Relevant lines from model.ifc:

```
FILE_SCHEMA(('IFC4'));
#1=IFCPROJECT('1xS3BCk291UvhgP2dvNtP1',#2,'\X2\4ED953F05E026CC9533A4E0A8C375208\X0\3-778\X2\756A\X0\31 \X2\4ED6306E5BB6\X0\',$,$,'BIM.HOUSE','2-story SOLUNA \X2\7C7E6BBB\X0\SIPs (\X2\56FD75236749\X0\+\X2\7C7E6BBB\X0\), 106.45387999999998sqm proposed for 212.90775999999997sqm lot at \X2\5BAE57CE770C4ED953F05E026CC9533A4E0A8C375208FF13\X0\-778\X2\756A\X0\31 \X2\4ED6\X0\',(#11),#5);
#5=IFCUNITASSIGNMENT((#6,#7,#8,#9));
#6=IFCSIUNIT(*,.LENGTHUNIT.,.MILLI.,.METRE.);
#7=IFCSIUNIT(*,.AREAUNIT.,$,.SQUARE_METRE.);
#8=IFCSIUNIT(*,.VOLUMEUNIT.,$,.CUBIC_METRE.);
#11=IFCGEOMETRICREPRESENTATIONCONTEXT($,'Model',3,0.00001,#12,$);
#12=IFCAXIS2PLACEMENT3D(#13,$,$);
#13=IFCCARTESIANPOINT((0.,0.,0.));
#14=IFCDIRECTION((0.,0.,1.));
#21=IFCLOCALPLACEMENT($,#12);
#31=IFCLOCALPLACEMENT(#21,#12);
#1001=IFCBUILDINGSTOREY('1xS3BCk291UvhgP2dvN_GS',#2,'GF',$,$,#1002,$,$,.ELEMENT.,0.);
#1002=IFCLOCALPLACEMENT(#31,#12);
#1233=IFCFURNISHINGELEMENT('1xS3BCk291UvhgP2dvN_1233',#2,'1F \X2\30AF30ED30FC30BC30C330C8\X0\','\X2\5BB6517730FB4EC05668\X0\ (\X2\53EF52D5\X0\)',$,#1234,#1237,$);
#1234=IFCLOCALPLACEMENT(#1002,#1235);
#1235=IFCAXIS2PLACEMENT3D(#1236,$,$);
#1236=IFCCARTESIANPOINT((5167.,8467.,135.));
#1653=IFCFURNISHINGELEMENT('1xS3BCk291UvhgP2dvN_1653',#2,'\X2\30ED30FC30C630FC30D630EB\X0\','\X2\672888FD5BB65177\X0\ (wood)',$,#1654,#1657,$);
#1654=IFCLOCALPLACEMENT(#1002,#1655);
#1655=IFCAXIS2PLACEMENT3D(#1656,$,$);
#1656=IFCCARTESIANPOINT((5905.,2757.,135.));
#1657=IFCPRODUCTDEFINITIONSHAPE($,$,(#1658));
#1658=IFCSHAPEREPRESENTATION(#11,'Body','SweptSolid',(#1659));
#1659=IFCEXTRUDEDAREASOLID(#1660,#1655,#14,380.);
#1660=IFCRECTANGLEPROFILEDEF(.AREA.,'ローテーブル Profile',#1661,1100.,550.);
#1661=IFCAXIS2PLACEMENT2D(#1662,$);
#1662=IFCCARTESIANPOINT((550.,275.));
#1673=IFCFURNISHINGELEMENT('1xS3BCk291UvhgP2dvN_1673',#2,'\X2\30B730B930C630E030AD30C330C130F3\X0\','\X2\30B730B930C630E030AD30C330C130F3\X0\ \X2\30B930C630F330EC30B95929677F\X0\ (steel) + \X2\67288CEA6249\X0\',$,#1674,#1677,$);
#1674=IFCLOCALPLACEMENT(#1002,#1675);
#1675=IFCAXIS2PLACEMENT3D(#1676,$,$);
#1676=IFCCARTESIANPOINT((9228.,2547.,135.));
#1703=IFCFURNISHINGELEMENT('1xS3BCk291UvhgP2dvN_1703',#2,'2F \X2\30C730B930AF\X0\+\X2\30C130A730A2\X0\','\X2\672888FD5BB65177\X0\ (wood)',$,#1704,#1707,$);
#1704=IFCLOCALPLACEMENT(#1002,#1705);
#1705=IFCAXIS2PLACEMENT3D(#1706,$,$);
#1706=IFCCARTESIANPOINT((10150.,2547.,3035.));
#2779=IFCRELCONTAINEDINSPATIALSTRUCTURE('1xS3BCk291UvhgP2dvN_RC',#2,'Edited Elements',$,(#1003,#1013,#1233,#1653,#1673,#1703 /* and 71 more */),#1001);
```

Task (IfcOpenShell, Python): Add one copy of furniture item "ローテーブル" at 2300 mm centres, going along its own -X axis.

```python
import ifcopenshell
import ifcopenshell.api.geometry
import ifcopenshell.api.root
import ifcopenshell.util.element
import ifcopenshell.util.placement
import ifcopenshell.util.unit

model = ifcopenshell.open("model.ifc")
unit_scale = ifcopenshell.util.unit.calculate_unit_scale(model)


def reuse_history(source, copy):
    """copy_class also copies each property set's owner history, people and application; keep the originals."""
    for rel in copy.IsDefinedBy:
        if rel.is_a("IfcRelDefinesByProperties") and (history := rel.RelatingPropertyDefinition.OwnerHistory):
            rel.RelatingPropertyDefinition.OwnerHistory = source.OwnerHistory
            ifcopenshell.util.element.remove_deep2(model, history)


source = model.by_guid("1xS3BCk291UvhgP2dvN_1653")
base = ifcopenshell.util.placement.get_local_placement(source.ObjectPlacement)
step = -base[:3, 0] * 2.3 / unit_scale

for i in range(1, 2):
    copy = ifcopenshell.api.root.copy_class(model, product=source)
    copy.Representation = ifcopenshell.util.element.copy_deep(
        model, source.Representation, exclude=["IfcGeometricRepresentationContext", "IfcRepresentationMap"]
    )
    reuse_history(source, copy)
    matrix = base.copy()
    matrix[:3, 3] += i * step
    print("added at", matrix[:3, 3].round(3) + 0.0)
    ifcopenshell.api.geometry.edit_object_placement(model, product=copy, matrix=matrix, is_si=False)

model.write("model-out.ifc")
```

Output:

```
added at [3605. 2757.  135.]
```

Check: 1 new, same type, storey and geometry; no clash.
